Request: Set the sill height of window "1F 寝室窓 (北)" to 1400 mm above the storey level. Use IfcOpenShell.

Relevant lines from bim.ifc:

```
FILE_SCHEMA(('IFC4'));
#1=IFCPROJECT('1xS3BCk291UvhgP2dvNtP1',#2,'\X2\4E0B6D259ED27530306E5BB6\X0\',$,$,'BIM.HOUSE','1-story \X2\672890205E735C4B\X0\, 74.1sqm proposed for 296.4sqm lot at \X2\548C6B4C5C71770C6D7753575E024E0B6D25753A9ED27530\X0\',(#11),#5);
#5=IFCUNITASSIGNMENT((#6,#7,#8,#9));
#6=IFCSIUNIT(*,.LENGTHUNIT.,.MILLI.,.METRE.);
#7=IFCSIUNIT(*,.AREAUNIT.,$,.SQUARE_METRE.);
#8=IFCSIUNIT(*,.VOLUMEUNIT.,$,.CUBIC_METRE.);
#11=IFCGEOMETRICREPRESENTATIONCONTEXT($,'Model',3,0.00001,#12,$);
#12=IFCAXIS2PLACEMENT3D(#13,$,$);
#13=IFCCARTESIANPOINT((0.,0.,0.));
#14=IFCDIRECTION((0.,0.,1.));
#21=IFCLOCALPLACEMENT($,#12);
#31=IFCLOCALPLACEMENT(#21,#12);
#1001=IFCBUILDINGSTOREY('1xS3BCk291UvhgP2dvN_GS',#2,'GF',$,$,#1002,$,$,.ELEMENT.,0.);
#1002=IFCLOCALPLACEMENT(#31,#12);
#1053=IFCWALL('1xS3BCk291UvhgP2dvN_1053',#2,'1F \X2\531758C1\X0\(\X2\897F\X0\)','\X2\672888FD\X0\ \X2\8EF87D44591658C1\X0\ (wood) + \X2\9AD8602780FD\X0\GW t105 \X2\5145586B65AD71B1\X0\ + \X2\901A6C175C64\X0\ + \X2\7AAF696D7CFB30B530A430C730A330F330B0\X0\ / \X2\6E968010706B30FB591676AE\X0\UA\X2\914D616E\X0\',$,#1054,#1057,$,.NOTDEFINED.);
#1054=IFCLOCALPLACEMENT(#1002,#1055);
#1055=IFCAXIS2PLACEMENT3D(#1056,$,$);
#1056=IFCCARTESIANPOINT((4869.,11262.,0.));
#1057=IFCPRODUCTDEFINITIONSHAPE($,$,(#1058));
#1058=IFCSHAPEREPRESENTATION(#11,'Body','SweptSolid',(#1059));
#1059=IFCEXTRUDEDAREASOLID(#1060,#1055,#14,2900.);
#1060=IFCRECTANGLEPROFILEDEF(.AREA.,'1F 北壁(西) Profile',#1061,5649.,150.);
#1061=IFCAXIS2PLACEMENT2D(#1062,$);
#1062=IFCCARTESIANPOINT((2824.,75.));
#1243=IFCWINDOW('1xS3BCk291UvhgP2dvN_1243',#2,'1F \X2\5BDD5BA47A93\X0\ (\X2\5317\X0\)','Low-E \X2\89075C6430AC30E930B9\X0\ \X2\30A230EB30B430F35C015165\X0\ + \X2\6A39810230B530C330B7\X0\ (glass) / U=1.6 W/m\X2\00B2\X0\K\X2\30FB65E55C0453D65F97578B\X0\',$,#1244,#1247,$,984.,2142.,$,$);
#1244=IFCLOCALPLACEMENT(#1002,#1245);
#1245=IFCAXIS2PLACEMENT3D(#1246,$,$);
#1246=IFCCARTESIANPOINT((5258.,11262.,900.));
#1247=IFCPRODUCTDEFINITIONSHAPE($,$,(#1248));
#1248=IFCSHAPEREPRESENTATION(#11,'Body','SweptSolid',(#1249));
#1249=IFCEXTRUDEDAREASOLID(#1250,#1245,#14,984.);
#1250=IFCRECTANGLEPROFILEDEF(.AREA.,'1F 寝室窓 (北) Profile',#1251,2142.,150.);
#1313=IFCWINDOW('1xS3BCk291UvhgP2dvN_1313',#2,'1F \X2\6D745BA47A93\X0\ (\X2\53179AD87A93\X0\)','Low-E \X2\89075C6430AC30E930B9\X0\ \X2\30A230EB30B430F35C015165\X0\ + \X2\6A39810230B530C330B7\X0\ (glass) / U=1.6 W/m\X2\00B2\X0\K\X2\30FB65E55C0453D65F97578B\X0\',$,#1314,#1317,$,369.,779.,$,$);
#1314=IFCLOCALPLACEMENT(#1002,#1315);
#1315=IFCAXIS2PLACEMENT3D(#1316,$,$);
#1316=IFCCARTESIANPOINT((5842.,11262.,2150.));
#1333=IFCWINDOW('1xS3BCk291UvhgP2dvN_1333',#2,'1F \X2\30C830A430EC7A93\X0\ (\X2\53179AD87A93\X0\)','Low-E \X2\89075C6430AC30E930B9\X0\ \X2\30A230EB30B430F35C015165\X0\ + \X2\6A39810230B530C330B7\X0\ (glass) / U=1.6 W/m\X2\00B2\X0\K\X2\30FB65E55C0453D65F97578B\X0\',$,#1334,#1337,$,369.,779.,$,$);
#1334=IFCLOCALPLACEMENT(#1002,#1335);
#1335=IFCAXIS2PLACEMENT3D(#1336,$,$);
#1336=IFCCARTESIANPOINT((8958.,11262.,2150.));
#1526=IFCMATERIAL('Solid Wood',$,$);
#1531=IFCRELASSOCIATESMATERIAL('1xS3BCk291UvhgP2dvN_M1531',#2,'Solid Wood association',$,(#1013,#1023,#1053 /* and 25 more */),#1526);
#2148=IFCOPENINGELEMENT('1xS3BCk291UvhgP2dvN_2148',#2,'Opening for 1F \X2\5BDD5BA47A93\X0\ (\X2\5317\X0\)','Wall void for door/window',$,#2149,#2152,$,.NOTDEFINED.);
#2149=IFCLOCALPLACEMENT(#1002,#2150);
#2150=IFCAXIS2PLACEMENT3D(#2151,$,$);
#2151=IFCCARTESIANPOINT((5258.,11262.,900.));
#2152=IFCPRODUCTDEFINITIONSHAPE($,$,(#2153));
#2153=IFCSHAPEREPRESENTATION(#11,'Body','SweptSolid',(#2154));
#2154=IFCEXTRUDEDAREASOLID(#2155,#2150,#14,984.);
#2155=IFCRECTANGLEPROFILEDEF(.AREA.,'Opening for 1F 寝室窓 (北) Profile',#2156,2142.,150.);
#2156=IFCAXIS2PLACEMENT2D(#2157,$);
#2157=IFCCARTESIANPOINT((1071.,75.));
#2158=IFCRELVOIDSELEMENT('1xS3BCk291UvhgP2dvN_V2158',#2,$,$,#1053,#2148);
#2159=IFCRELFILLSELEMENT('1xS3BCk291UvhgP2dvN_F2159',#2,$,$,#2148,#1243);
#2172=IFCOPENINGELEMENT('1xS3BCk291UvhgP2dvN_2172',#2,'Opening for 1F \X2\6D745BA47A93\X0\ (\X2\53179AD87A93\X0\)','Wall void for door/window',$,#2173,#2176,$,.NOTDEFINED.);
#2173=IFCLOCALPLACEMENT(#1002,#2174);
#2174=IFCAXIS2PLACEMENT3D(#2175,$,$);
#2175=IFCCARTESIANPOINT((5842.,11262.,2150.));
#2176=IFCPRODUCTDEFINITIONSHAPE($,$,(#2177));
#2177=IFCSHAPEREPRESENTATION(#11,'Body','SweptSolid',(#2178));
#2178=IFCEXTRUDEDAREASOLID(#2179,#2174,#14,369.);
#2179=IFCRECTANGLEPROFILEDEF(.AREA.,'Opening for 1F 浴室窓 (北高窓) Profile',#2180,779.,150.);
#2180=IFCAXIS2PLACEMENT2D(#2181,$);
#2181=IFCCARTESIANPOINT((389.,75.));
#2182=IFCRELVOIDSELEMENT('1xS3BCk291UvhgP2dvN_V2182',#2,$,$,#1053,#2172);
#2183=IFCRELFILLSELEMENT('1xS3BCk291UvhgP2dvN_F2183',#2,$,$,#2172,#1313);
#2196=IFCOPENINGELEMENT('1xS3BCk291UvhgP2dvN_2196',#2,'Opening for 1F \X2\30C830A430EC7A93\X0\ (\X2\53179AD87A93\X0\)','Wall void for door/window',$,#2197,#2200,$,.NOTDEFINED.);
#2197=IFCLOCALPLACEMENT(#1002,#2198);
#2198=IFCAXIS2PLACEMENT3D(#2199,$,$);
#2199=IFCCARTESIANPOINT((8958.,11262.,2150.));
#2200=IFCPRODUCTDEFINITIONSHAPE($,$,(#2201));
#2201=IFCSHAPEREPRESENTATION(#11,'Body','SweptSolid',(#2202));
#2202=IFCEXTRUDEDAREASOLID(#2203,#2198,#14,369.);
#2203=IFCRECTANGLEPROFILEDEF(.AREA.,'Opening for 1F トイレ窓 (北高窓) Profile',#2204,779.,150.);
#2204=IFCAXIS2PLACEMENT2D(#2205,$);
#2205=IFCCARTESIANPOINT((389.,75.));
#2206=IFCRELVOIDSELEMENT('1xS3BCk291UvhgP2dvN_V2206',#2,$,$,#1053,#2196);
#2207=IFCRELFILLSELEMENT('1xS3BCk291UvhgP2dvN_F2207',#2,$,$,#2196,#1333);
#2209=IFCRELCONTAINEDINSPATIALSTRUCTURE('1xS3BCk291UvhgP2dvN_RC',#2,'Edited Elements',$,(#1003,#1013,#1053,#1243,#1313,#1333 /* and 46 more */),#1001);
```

```python
import numpy as np
import ifcopenshell
import ifcopenshell.api.geometry
import ifcopenshell.geom
import ifcopenshell.util.element
import ifcopenshell.util.placement
import ifcopenshell.util.shape
import ifcopenshell.util.unit

model = ifcopenshell.open("bim.ifc")
unit_scale = ifcopenshell.util.unit.calculate_unit_scale(model)

window = model.by_guid("1xS3BCk291UvhgP2dvN_1243")
opening = window.FillsVoids[0].RelatingOpeningElement
storey = ifcopenshell.util.element.get_container(window, ifc_class="IfcBuildingStorey")
level = ifcopenshell.util.placement.get_local_placement(storey.ObjectPlacement)[2, 3]

# The opening's origin need not be at the sill, so measure its lowest point.
shape = ifcopenshell.geom.create_shape(ifcopenshell.geom.settings(), opening)
bottom = ifcopenshell.util.shape.get_shape_bottom_elevation(shape, shape.geometry) / unit_scale
dz = level + 1400.0 - bottom

shift = np.array([0.0, 0.0, dz])
# The window is not placed relative to its opening, so move both.
for product in (opening, window):
    matrix = ifcopenshell.util.placement.get_local_placement(product.ObjectPlacement)
    matrix[:3, 3] += shift
    ifcopenshell.api.geometry.edit_object_placement(model, product=product, matrix=matrix, is_si=False)

print(f"moved by {dz * unit_scale:+.3f} m")

model.write("bim_updated.ifc")
```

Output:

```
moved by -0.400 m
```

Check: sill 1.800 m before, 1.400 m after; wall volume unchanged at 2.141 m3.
